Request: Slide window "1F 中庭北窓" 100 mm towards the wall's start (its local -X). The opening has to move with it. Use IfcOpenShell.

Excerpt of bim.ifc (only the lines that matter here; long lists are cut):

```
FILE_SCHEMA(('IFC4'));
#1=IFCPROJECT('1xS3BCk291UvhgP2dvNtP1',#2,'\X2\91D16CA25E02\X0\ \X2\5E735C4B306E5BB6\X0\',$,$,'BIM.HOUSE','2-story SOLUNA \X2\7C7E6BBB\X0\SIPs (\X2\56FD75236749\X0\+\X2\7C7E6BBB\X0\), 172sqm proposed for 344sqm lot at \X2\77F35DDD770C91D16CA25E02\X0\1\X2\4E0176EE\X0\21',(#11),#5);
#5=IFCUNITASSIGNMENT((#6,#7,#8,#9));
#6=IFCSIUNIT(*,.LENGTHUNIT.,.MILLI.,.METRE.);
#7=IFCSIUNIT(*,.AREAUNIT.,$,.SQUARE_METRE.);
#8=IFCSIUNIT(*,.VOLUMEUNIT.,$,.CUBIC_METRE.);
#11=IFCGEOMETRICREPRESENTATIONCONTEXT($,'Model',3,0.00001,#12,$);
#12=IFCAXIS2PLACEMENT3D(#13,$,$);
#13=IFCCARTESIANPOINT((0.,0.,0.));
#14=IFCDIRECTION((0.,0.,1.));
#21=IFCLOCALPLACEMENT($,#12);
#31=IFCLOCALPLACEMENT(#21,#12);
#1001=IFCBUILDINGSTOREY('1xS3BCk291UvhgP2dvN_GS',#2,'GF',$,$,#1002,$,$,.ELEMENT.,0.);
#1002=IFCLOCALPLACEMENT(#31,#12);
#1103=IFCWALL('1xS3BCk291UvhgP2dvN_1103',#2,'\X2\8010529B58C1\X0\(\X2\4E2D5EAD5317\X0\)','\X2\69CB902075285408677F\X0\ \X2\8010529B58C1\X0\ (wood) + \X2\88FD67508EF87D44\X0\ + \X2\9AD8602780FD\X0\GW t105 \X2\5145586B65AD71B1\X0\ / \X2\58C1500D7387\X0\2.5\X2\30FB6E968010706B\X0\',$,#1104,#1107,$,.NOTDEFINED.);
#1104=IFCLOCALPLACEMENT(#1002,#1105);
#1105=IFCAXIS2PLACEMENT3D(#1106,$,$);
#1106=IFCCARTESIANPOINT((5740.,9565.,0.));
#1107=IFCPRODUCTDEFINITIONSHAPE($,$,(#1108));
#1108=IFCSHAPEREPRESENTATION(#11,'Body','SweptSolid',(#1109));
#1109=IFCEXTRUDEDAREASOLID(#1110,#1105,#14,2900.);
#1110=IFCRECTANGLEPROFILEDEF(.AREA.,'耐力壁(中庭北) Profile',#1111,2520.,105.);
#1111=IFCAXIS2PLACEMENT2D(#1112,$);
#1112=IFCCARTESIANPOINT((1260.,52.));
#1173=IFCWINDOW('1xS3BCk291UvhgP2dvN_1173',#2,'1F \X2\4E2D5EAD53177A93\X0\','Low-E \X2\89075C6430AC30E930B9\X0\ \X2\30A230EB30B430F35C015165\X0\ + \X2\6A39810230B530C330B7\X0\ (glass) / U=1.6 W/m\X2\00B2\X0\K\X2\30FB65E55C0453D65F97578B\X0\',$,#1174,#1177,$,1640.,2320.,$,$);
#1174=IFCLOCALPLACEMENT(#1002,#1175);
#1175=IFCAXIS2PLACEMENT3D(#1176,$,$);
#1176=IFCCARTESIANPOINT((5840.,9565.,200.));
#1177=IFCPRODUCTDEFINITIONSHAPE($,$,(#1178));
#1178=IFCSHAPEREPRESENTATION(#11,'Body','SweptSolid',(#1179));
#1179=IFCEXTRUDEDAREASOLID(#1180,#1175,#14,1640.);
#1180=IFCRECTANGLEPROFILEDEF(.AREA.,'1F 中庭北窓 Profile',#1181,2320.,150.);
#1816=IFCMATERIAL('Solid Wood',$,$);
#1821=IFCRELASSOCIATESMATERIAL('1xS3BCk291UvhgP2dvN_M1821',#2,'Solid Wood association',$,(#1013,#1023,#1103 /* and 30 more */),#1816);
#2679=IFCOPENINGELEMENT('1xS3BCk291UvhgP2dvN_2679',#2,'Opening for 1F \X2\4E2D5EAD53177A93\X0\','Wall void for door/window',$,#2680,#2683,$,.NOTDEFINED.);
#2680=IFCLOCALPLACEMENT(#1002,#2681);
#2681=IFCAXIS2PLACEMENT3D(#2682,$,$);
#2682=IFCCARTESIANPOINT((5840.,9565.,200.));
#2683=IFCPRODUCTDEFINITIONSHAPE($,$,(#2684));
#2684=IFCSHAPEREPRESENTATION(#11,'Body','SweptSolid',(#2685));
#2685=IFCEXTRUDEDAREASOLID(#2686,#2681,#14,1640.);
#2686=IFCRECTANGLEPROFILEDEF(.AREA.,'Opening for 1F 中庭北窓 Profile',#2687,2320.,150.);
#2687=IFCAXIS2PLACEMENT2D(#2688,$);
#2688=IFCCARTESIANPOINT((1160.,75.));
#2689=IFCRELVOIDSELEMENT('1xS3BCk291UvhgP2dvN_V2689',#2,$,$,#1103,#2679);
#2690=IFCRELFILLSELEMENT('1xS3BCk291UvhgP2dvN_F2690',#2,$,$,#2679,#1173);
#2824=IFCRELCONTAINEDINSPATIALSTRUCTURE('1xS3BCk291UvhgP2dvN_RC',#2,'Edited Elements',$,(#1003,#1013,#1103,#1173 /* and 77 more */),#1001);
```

```python
import ifcopenshell
import ifcopenshell.api.geometry
import ifcopenshell.util.placement
import ifcopenshell.util.unit

model = ifcopenshell.open("bim.ifc")
unit_scale = ifcopenshell.util.unit.calculate_unit_scale(model)

window = model.by_guid("1xS3BCk291UvhgP2dvN_1173")
opening = window.FillsVoids[0].RelatingOpeningElement
wall = opening.VoidsElements[0].RelatingBuildingElement

wall_matrix = ifcopenshell.util.placement.get_local_placement(wall.ObjectPlacement)
shift = wall_matrix[:3, 0] * -0.1 / unit_scale
before = ifcopenshell.util.placement.get_local_placement(window.ObjectPlacement)[:3, 3].copy()

# The window is not placed relative to its opening, so move both.
for product in (opening, window):
    matrix = ifcopenshell.util.placement.get_local_placement(product.ObjectPlacement)
    matrix[:3, 3] += shift
    ifcopenshell.api.geometry.edit_object_placement(model, product=product, matrix=matrix, is_si=False)

after = ifcopenshell.util.placement.get_local_placement(window.ObjectPlacement)[:3, 3]
print("window moved by", (after - before).round(3) + 0.0)

model.write("bim_rev.ifc")
```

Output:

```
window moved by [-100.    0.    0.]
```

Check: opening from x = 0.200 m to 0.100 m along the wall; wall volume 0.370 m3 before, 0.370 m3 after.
